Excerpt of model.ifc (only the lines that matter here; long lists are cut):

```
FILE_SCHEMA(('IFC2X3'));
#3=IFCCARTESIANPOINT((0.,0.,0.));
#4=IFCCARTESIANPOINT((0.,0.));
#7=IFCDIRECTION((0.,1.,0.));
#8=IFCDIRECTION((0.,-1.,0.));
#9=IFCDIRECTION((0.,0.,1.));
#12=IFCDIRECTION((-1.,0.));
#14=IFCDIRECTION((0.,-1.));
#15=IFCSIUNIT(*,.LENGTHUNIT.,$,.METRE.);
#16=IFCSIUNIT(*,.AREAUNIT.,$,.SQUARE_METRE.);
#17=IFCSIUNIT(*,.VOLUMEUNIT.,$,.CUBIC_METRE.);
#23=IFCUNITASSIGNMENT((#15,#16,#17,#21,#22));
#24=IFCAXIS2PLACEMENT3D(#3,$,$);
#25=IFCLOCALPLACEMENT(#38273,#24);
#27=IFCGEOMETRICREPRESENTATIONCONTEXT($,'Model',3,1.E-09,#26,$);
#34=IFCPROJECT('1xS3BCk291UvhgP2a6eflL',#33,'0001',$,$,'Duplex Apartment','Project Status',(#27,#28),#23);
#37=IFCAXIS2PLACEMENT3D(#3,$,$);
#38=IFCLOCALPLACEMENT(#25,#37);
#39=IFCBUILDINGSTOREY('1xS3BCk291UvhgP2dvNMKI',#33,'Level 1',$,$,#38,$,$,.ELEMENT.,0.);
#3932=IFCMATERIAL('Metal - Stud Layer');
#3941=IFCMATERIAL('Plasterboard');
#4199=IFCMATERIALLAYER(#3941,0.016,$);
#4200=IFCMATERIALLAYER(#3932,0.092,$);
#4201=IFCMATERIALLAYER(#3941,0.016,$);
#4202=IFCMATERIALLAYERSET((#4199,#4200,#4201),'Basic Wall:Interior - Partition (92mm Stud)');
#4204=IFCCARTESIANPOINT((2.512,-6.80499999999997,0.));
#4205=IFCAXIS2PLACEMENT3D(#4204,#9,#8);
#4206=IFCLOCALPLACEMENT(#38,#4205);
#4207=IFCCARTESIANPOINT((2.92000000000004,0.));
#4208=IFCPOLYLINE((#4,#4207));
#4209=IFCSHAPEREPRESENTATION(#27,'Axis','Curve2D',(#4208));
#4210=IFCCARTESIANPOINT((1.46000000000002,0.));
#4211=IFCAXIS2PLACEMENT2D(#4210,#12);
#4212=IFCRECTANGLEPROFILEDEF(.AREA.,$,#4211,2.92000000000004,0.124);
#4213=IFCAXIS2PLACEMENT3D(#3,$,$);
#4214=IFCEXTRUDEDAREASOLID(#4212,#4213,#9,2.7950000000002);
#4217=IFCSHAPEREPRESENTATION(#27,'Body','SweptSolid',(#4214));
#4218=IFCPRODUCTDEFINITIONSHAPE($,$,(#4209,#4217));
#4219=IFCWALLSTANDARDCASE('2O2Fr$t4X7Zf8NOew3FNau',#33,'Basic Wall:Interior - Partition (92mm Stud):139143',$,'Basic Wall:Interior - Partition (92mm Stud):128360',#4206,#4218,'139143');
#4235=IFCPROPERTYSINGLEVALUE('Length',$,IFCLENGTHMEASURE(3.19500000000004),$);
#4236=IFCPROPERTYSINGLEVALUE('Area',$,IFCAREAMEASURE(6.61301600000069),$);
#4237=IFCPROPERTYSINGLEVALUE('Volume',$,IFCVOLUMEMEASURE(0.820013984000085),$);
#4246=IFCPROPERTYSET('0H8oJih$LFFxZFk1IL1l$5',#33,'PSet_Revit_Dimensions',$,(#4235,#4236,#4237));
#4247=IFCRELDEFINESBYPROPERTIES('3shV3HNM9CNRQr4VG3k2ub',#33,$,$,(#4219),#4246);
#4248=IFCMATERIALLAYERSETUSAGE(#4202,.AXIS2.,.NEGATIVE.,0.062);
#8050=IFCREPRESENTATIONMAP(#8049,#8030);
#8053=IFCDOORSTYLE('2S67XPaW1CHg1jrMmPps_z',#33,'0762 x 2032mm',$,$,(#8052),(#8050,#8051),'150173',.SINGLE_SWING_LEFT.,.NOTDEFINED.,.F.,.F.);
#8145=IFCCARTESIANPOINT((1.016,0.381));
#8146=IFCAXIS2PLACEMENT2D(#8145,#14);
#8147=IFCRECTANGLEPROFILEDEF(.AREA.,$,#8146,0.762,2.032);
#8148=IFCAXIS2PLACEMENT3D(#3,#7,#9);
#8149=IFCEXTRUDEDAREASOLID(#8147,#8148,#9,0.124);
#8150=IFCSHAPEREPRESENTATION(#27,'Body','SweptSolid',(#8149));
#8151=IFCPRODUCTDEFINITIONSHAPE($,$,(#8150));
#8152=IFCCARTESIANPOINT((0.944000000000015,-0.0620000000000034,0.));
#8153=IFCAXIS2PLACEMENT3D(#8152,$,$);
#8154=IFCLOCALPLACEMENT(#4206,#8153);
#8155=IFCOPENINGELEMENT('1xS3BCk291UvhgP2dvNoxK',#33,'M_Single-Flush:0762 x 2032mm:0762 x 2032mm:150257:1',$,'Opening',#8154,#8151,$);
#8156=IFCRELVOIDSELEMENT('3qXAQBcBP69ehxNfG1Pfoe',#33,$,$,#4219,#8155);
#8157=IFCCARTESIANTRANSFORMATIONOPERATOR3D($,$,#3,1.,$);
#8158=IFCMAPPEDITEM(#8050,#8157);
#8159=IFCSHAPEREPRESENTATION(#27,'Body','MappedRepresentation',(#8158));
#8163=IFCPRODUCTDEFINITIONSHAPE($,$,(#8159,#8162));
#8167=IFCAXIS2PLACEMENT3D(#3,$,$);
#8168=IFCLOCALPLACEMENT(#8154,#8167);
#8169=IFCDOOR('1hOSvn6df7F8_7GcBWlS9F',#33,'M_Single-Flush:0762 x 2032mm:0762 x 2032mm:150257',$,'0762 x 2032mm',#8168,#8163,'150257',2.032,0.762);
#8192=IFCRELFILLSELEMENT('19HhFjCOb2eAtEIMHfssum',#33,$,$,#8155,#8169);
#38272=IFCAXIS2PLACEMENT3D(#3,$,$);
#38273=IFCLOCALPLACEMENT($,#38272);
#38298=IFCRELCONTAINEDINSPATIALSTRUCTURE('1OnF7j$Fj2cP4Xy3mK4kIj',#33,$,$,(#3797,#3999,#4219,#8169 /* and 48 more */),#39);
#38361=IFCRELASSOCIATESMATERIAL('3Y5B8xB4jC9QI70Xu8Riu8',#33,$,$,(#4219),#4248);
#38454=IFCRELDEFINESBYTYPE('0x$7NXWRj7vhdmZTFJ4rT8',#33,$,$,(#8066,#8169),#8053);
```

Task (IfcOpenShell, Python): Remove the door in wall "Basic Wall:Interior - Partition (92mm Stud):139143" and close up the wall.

```python
import ifcopenshell
import ifcopenshell.api.feature
import ifcopenshell.api.pset
import ifcopenshell.api.root
import ifcopenshell.geom
import ifcopenshell.util.element
import ifcopenshell.util.shape
import ifcopenshell.util.unit

model = ifcopenshell.open("model.ifc")
area_scale = ifcopenshell.util.unit.calculate_unit_scale(model, "AREAUNIT")
volume_scale = ifcopenshell.util.unit.calculate_unit_scale(model, "VOLUMEUNIT")
settings = ifcopenshell.geom.settings()


def volume(element):
    """Net volume in cubic metres, openings subtracted."""
    shape = ifcopenshell.geom.create_shape(settings, element)
    return ifcopenshell.util.shape.get_volume(shape.geometry)


door = model.by_id(8169)
opening = door.FillsVoids[0].RelatingOpeningElement
wall = opening.VoidsElements[0].RelatingBuildingElement
before = volume(wall)

ifcopenshell.api.root.remove_product(model, product=door)
ifcopenshell.api.feature.remove_feature(model, feature=opening)

after = volume(wall)
thickness = 0.124  # wall thickness in metres

# Update the wall's stored quantities.
pset = model.by_id(ifcopenshell.util.element.get_pset(wall, "PSet_Revit_Dimensions", should_inherit=False)["id"])
ifcopenshell.api.pset.edit_pset(model, pset=pset, properties={
    "Area": model.create_entity("IfcAreaMeasure", after / thickness / area_scale),
    "Volume": model.create_entity("IfcVolumeMeasure", after / volume_scale),
})

print(f"wall volume {before:.3f} -> {after:.3f} m3")

model.write("model_updated.ifc")
```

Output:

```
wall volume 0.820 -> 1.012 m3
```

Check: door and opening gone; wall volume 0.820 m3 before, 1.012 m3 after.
